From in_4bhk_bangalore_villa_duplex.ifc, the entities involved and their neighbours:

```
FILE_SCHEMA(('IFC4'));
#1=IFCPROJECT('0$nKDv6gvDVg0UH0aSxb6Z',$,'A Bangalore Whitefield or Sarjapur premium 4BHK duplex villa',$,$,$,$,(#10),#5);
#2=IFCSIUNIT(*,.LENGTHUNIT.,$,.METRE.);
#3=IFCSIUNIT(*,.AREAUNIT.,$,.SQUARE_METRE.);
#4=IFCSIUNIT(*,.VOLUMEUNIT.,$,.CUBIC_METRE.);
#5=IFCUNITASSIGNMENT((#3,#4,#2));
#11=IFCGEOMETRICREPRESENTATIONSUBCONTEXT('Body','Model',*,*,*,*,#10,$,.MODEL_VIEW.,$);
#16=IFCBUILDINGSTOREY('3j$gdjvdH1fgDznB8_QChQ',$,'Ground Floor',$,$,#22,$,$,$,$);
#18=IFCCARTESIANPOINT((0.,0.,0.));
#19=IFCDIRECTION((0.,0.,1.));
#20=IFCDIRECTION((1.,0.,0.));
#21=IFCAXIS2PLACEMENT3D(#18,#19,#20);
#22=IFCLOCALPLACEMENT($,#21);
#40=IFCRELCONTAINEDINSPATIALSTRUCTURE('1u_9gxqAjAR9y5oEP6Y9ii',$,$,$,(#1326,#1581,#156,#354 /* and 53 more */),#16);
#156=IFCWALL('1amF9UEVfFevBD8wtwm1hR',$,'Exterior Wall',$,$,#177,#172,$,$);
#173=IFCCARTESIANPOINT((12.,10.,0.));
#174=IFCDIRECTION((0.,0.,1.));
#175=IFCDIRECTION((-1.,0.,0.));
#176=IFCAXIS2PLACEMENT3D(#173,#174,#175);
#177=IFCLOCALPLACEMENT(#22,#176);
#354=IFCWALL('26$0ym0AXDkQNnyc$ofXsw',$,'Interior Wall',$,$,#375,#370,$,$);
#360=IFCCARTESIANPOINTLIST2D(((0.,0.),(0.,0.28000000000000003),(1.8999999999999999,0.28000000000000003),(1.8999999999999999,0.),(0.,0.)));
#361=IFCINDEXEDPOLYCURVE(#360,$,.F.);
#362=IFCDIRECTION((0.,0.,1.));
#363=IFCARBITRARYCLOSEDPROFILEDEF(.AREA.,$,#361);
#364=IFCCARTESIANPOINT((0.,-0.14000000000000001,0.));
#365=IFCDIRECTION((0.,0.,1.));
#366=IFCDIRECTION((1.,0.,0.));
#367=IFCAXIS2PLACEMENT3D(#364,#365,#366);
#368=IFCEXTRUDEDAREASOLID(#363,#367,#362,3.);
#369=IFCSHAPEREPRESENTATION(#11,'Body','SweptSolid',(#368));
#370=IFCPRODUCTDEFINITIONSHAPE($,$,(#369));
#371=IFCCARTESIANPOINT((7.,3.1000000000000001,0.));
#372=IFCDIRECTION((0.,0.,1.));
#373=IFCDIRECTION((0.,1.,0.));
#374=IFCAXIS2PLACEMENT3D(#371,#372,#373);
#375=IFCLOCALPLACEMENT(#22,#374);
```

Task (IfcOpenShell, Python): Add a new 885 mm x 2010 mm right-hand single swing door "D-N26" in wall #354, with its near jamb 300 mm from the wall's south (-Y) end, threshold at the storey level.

```python
import numpy as np
import ifcopenshell
import ifcopenshell.api.feature
import ifcopenshell.api.geometry
import ifcopenshell.api.root
import ifcopenshell.api.spatial
import ifcopenshell.geom
import ifcopenshell.util.element
import ifcopenshell.util.placement
import ifcopenshell.util.representation
import ifcopenshell.util.shape
import ifcopenshell.util.unit

model = ifcopenshell.open("in_4bhk_bangalore_villa_duplex.ifc")
unit_scale = ifcopenshell.util.unit.calculate_unit_scale(model)
settings = ifcopenshell.geom.settings()


def volume(element):
    """Net volume in cubic metres, openings subtracted."""
    shape = ifcopenshell.geom.create_shape(settings, element)
    return ifcopenshell.util.shape.get_volume(shape.geometry)


wall = model.by_guid("26$0ym0AXDkQNnyc$ofXsw")
storey = ifcopenshell.util.element.get_container(wall, ifc_class="IfcBuildingStorey")
context = ifcopenshell.util.representation.get_context(model, "Model", "Body", "MODEL_VIEW")
before = volume(wall)

width, height, from_end, sill = 0.885, 2.01, 0.3, 0.0  # metres

# The wall runs along its own X axis, and the end named is its -X end.
wall_shape = ifcopenshell.geom.create_shape(settings, wall)
x, y, z = ifcopenshell.util.shape.get_vertices(wall_shape.geometry).T
start = x.min() + from_end
face, thickness = float(y.min()), float(y.max() - y.min())
wall_matrix = ifcopenshell.util.placement.get_local_placement(wall.ObjectPlacement)
level = ifcopenshell.util.placement.get_local_placement(storey.ObjectPlacement)[2, 3]


def in_wall(x, y):
    """Placement at x, y metres in the wall's axes, at sill height."""
    matrix = wall_matrix.copy()
    matrix[:, 3] = wall_matrix @ np.array([x / unit_scale, y / unit_scale, 0.0, 1.0])
    matrix[2, 3] = level + sill / unit_scale
    return matrix


# Opening: a box that overshoots both wall faces by 50 mm.
opening = ifcopenshell.api.root.create_entity(model, ifc_class="IfcOpeningElement", predefined_type="OPENING")
box = ifcopenshell.api.geometry.add_wall_representation(
    model, context=context, length=width, height=height, thickness=thickness + 0.1
)
ifcopenshell.api.geometry.assign_representation(model, product=opening, representation=box)
ifcopenshell.api.geometry.edit_object_placement(model, product=opening, matrix=in_wall(start, face - 0.05), is_si=False)
ifcopenshell.api.feature.add_feature(model, feature=opening, element=wall)

door = ifcopenshell.api.root.create_entity(model, ifc_class="IfcDoor", name="D-N26", predefined_type="DOOR")
door.OverallWidth, door.OverallHeight = width / unit_scale, height / unit_scale
door.OperationType = "SINGLE_SWING_RIGHT"
body = ifcopenshell.api.geometry.add_door_representation(
    model,
    context=context,
    overall_width=door.OverallWidth,
    overall_height=door.OverallHeight,
    operation_type="SINGLE_SWING_RIGHT",
    lining_properties={"LiningDepth": thickness / unit_scale, "ThresholdDepth": thickness / unit_scale},
)
ifcopenshell.api.geometry.assign_representation(model, product=door, representation=body)
ifcopenshell.api.spatial.assign_container(model, products=[door], relating_structure=storey)
ifcopenshell.api.feature.add_filling(model, opening=opening, element=door)

# The lining spans the wall, so the door starts at the wall face.
ifcopenshell.api.geometry.edit_object_placement(model, product=door, matrix=in_wall(start, face), is_si=False)

after = volume(wall)

print(f"wall volume {before:.3f} -> {after:.3f} m3")

model.write("in_4bhk_bangalore_villa_duplex_edited.ifc")
```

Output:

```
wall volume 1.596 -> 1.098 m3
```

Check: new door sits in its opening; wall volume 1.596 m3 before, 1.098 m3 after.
